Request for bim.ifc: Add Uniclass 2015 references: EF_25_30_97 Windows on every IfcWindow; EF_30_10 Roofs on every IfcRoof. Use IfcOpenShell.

First a look at what the model holds.

```python
import ifcopenshell

model = ifcopenshell.open("bim.ifc")
print(model.schema)
print("classifications:", [c.Name for c in model.by_type("IfcClassification")])
for ifc_class in ("IfcDoor", "IfcRoof", "IfcStair", "IfcWall", "IfcWindow"):
    print(ifc_class, len(model.by_type(ifc_class)))
```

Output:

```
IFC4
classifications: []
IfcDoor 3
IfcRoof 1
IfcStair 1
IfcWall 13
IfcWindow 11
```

```python
import ifcopenshell
import ifcopenshell.api.classification

model = ifcopenshell.open("bim.ifc")

system = ifcopenshell.api.classification.add_classification(model, classification="Uniclass 2015")

codes = {
    "IfcWindow": ("EF_25_30_97", "Windows"),
    "IfcRoof": ("EF_30_10", "Roofs"),
}
for ifc_class, (code, name) in codes.items():
    products = model.by_type(ifc_class)
    ifcopenshell.api.classification.add_reference(
        model, products=products, classification=system, identification=code, name=name
    )
    print(code, len(products))

model.write("bim-out.ifc")
```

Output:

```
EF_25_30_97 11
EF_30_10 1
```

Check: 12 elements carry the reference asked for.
